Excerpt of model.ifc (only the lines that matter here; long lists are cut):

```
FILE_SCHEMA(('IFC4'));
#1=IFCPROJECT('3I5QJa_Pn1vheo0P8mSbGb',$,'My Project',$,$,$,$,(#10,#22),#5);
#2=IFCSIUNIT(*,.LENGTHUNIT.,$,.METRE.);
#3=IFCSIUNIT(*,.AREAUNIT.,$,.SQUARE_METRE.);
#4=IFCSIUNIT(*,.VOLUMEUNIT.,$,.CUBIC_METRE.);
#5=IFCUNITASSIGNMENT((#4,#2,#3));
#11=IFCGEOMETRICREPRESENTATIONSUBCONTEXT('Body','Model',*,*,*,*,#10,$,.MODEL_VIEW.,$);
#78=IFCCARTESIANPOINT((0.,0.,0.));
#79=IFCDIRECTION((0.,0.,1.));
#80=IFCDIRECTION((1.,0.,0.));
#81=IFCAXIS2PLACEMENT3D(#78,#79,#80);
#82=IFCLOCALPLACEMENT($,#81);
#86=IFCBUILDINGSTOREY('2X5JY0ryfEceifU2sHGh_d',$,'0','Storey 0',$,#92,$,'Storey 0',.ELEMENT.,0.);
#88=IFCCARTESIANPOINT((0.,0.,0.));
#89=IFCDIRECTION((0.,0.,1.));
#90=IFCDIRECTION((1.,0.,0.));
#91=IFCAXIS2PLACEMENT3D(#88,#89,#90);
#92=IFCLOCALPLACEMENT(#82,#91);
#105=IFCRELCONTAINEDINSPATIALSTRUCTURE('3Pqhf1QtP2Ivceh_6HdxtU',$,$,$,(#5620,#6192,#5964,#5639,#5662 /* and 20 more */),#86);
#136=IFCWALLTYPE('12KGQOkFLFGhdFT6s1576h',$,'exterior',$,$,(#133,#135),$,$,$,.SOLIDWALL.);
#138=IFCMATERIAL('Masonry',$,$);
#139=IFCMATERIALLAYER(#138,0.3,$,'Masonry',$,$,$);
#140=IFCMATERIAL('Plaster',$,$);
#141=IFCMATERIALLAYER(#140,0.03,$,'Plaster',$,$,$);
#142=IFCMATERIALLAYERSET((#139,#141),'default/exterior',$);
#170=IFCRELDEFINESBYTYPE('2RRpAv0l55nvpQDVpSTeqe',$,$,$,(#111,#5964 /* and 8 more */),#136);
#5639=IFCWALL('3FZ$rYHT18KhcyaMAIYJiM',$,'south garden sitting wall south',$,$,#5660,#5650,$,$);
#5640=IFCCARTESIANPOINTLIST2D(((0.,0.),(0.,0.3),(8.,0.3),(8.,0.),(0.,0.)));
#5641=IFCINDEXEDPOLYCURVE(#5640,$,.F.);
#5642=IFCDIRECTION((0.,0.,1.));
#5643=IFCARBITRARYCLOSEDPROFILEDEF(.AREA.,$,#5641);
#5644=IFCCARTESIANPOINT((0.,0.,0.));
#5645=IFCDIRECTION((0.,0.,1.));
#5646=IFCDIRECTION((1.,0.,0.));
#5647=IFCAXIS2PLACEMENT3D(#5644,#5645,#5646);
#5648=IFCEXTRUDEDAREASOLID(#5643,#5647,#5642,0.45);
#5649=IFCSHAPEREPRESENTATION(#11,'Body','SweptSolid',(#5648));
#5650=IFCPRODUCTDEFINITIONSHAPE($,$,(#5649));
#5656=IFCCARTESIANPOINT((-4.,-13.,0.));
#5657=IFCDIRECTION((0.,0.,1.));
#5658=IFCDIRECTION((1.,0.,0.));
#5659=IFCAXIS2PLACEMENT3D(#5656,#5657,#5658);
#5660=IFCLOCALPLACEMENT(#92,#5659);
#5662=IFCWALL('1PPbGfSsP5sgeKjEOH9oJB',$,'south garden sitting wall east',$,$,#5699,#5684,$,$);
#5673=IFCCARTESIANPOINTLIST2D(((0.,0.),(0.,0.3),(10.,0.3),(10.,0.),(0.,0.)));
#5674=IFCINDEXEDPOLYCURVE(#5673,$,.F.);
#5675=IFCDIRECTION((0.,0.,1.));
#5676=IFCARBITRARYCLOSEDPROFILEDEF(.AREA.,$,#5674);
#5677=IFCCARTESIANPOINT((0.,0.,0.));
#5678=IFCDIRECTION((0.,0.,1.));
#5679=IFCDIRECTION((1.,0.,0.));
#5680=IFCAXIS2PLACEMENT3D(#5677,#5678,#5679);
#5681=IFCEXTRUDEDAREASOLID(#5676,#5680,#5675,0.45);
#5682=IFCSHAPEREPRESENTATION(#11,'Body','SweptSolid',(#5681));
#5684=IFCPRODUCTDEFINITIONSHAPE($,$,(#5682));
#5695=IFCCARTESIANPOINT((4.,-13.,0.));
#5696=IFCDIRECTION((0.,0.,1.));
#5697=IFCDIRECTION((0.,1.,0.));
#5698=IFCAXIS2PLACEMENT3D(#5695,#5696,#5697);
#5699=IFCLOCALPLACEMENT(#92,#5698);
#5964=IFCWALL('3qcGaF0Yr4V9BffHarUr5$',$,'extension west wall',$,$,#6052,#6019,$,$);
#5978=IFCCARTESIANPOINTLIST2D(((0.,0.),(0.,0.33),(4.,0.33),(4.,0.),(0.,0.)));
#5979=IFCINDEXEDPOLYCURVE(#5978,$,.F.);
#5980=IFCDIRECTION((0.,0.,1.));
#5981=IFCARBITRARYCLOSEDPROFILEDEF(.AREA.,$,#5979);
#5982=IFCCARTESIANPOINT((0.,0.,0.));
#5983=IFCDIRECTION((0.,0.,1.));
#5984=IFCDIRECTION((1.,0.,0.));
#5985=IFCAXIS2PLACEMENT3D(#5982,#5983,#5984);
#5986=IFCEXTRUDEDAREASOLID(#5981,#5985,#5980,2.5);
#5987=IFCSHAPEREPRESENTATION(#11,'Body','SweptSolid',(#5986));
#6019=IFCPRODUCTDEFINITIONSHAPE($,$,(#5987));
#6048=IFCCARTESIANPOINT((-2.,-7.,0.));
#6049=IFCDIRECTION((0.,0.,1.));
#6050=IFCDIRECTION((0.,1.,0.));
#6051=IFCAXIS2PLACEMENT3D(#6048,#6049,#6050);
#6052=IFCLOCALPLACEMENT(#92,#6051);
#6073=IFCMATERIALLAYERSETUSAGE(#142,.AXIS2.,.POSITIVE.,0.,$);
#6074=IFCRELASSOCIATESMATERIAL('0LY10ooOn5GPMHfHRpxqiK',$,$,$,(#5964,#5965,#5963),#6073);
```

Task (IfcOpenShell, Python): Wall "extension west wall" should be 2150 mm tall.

```python
import ifcopenshell
import ifcopenshell.geom
import ifcopenshell.util.representation
import ifcopenshell.util.shape

model = ifcopenshell.open("model.ifc")
settings = ifcopenshell.geom.settings()


def volume(element):
    """Net volume in cubic metres, openings subtracted."""
    shape = ifcopenshell.geom.create_shape(settings, element)
    return ifcopenshell.util.shape.get_volume(shape.geometry)


wall = model.by_guid("3qcGaF0Yr4V9BffHarUr5$")
before = volume(wall)

body = ifcopenshell.util.representation.get_representation(wall, "Model", "Body")
solid = body.Items[0]
old_height = solid.Depth
solid.Depth = 2.15
after = volume(wall)

print(f"height {old_height:g} -> {solid.Depth:g}, volume {before:.3f} -> {after:.3f} m3")

model.write("model_rev.ifc")
```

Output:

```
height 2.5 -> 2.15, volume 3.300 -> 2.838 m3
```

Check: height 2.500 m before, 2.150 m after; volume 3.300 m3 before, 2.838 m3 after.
